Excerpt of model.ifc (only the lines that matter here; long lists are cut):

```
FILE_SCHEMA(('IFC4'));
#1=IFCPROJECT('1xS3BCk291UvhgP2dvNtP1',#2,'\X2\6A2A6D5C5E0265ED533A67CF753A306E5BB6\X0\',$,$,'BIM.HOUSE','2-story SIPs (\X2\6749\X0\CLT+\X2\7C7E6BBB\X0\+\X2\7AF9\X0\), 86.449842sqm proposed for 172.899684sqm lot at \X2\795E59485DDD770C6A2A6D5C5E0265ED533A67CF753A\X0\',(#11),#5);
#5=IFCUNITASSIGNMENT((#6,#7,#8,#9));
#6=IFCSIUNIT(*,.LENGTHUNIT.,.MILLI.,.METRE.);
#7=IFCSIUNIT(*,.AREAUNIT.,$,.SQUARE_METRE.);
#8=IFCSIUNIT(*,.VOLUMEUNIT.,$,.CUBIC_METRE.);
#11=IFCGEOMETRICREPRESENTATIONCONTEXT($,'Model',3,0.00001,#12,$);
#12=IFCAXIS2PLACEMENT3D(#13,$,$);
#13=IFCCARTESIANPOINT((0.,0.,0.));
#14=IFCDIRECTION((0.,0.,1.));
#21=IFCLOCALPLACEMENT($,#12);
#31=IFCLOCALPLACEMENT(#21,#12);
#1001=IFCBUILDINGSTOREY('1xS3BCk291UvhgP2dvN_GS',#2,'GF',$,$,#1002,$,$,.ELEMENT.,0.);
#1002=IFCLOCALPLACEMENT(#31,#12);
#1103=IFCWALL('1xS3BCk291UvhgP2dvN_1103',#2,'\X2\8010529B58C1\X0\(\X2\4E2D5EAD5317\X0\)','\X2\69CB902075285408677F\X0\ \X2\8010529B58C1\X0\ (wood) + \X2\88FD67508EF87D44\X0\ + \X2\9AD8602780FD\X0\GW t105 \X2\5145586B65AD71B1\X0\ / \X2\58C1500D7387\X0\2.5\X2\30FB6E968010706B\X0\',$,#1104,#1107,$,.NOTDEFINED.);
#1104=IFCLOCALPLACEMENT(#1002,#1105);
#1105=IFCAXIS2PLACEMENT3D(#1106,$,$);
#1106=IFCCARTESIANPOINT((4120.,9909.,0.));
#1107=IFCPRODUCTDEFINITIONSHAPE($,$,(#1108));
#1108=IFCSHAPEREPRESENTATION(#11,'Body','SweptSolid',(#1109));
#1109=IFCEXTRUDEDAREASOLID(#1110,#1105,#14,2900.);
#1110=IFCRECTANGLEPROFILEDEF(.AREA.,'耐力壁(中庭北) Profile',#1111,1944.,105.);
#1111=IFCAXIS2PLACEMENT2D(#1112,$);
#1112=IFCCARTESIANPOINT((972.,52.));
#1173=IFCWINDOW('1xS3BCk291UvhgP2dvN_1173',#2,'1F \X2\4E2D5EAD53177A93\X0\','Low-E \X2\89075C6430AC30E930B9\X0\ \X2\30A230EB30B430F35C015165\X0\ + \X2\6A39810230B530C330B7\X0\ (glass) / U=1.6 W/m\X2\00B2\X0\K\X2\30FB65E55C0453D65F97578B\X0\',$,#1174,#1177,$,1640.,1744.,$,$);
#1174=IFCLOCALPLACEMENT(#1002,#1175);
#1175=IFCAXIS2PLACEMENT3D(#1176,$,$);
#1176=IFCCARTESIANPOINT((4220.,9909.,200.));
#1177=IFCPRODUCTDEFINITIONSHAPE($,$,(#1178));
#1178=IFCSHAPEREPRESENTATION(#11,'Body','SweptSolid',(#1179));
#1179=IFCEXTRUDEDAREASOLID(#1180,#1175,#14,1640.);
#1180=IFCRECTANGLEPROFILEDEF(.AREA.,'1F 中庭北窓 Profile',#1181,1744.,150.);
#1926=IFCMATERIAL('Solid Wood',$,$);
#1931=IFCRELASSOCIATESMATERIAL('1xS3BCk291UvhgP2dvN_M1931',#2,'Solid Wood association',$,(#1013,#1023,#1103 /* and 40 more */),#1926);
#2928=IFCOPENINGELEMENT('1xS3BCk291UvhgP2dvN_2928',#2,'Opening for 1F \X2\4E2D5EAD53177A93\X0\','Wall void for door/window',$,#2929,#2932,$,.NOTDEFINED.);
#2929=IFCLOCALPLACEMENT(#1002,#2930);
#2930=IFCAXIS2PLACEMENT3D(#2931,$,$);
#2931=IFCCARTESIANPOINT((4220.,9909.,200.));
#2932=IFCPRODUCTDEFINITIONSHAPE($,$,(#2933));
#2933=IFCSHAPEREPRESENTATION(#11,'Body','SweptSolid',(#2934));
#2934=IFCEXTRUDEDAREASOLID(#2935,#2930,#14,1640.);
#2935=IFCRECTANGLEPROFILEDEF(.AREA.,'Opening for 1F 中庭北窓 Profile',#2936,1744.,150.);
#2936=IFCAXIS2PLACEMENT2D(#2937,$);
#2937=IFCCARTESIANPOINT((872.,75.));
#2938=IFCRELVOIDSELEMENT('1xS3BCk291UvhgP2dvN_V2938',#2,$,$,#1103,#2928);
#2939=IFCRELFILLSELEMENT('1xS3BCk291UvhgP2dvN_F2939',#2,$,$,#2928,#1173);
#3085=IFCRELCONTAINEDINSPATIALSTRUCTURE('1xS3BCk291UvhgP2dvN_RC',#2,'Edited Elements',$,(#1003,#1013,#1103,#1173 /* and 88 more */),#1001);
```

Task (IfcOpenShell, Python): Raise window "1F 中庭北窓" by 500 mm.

```python
import numpy as np
import ifcopenshell
import ifcopenshell.api.geometry
import ifcopenshell.util.placement
import ifcopenshell.util.unit

model = ifcopenshell.open("model.ifc")
unit_scale = ifcopenshell.util.unit.calculate_unit_scale(model)

window = model.by_guid("1xS3BCk291UvhgP2dvN_1173")
opening = window.FillsVoids[0].RelatingOpeningElement
dz = 500.0

shift = np.array([0.0, 0.0, dz])
# The window is not placed relative to its opening, so move both.
for product in (opening, window):
    matrix = ifcopenshell.util.placement.get_local_placement(product.ObjectPlacement)
    matrix[:3, 3] += shift
    ifcopenshell.api.geometry.edit_object_placement(model, product=product, matrix=matrix, is_si=False)

print(f"moved by {dz * unit_scale:+.3f} m")

model.write("model_edited.ifc")
```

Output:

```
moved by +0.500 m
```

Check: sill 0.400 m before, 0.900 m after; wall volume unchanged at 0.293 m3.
